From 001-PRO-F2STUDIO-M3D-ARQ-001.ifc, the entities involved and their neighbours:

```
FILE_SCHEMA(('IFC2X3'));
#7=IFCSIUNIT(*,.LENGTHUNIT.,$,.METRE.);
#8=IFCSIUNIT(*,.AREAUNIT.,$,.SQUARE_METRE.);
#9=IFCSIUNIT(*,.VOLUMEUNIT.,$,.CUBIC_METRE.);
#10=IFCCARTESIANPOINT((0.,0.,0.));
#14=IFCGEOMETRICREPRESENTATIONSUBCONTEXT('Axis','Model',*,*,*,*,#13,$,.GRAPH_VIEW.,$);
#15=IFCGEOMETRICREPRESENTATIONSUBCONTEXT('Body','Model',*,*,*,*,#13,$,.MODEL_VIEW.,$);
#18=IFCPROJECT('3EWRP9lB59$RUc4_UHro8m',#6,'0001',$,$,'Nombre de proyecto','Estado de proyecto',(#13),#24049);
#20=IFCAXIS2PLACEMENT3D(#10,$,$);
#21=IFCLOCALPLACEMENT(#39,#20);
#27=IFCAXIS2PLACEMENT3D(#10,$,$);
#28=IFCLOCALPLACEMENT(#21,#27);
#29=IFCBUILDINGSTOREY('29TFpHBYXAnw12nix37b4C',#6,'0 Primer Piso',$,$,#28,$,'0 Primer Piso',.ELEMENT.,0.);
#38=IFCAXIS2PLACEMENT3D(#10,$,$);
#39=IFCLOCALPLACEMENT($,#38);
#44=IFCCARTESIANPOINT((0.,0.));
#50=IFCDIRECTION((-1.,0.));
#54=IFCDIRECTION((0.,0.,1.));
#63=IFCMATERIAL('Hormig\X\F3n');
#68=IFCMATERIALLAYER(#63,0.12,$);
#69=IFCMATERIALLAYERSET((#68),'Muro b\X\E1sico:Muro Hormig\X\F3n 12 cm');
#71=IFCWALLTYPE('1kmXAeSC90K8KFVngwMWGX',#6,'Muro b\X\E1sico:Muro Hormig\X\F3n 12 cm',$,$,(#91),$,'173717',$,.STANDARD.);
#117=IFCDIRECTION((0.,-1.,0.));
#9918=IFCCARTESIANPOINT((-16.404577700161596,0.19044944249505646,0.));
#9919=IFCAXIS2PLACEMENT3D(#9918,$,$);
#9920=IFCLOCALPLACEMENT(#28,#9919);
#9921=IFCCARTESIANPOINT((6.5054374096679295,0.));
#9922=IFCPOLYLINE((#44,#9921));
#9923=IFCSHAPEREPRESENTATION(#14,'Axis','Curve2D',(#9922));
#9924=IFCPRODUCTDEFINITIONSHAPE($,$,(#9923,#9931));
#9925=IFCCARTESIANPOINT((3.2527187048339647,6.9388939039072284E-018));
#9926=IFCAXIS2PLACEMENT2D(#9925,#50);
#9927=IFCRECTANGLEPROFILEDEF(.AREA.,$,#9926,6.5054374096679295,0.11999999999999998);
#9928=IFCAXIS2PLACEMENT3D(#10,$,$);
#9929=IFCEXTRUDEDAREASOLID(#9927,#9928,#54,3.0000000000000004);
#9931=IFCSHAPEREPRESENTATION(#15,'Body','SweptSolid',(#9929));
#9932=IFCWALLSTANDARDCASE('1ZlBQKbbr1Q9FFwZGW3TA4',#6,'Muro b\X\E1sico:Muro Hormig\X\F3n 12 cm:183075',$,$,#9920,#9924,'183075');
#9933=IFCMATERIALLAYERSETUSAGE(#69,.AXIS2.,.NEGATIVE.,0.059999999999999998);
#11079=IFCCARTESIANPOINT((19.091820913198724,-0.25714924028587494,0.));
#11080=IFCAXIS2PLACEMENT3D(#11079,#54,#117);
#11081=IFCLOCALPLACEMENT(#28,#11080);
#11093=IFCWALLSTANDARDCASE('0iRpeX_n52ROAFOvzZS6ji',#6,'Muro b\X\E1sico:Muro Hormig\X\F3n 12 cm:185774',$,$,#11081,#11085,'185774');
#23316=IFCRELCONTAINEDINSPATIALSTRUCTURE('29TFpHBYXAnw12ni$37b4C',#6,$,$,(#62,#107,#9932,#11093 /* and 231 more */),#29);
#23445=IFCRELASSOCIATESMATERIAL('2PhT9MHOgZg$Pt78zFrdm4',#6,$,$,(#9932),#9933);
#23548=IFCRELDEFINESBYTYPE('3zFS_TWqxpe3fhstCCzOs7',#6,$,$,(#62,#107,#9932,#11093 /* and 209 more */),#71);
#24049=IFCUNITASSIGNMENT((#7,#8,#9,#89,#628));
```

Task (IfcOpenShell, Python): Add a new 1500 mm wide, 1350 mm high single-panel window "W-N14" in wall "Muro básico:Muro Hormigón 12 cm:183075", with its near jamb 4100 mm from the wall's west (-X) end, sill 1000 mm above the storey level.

```python
import numpy as np
import ifcopenshell
import ifcopenshell.api.feature
import ifcopenshell.api.geometry
import ifcopenshell.api.root
import ifcopenshell.api.spatial
import ifcopenshell.api.type
import ifcopenshell.geom
import ifcopenshell.util.element
import ifcopenshell.util.placement
import ifcopenshell.util.representation
import ifcopenshell.util.shape
import ifcopenshell.util.unit

model = ifcopenshell.open("001-PRO-F2STUDIO-M3D-ARQ-001.ifc")
unit_scale = ifcopenshell.util.unit.calculate_unit_scale(model)
settings = ifcopenshell.geom.settings()


def volume(element):
    """Net volume in cubic metres, openings subtracted."""
    shape = ifcopenshell.geom.create_shape(settings, element)
    return ifcopenshell.util.shape.get_volume(shape.geometry)


wall = model.by_guid("1ZlBQKbbr1Q9FFwZGW3TA4")
storey = ifcopenshell.util.element.get_container(wall, ifc_class="IfcBuildingStorey")
context = ifcopenshell.util.representation.get_context(model, "Model", "Body", "MODEL_VIEW")
before = volume(wall)

width, height, from_end, sill = 1.5, 1.35, 4.1, 1  # metres

# The wall runs along its own X axis, and the end named is its -X end.
wall_shape = ifcopenshell.geom.create_shape(settings, wall)
x, y, z = ifcopenshell.util.shape.get_vertices(wall_shape.geometry).T
start = x.min() + from_end
face, thickness = float(y.min()), float(y.max() - y.min())
wall_matrix = ifcopenshell.util.placement.get_local_placement(wall.ObjectPlacement)
level = ifcopenshell.util.placement.get_local_placement(storey.ObjectPlacement)[2, 3]


def in_wall(x, y):
    """Placement at x, y metres in the wall's axes, at sill height."""
    matrix = wall_matrix.copy()
    matrix[:, 3] = wall_matrix @ np.array([x / unit_scale, y / unit_scale, 0.0, 1.0])
    matrix[2, 3] = level + sill / unit_scale
    return matrix


# Opening: a box that overshoots both wall faces by 50 mm.
opening = ifcopenshell.api.root.create_entity(model, ifc_class="IfcOpeningElement")
box = ifcopenshell.api.geometry.add_wall_representation(
    model, context=context, length=width, height=height, thickness=thickness + 0.1
)
ifcopenshell.api.geometry.assign_representation(model, product=opening, representation=box)
ifcopenshell.api.geometry.edit_object_placement(model, product=opening, matrix=in_wall(start, face - 0.05), is_si=False)
ifcopenshell.api.feature.add_feature(model, feature=opening, element=wall)

window = ifcopenshell.api.root.create_entity(model, ifc_class="IfcWindow", name="W-N14")
window.OverallWidth, window.OverallHeight = width / unit_scale, height / unit_scale
body = ifcopenshell.api.geometry.add_window_representation(
    model,
    context=context,
    overall_width=window.OverallWidth,
    overall_height=window.OverallHeight,
    partition_type="SINGLE_PANEL",
)
ifcopenshell.api.geometry.assign_representation(model, product=window, representation=body)
ifcopenshell.api.spatial.assign_container(model, products=[window], relating_structure=storey)
fills = ifcopenshell.api.feature.add_filling(model, opening=opening, element=window)
fills.OwnerHistory = window.OwnerHistory  # required in IFC2X3

# IFC2X3 keeps the operation on the window style.
style = ifcopenshell.api.root.create_entity(model, ifc_class="IfcWindowStyle", name="W-N14")
style.OperationType, style.ConstructionType = "SINGLE_PANEL", "NOTDEFINED"
style.ParameterTakesPrecedence = style.Sizeable = False
ifcopenshell.api.type.assign_type(model, related_objects=[window], relating_type=style)

# Centre the window in the wall's thickness.
ifcopenshell.api.geometry.edit_object_placement(model, product=window, matrix=in_wall(start, face), is_si=False)
window_shape = ifcopenshell.geom.create_shape(settings, window)
depth = ifcopenshell.util.shape.get_vertices(window_shape.geometry)[:, 1]
offset = face + thickness / 2 - (depth.min() + depth.max()) / 2
ifcopenshell.api.geometry.edit_object_placement(model, product=window, matrix=in_wall(start, offset), is_si=False)

after = volume(wall)

print(f"wall volume {before:.3f} -> {after:.3f} m3")

model.write("001-PRO-F2STUDIO-M3D-ARQ-001_v2.ifc")
```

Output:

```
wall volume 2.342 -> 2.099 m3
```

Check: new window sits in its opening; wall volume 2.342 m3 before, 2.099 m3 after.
